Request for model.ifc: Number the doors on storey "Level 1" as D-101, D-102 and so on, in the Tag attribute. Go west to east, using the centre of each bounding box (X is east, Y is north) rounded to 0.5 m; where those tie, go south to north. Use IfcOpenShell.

First a look at what the model holds.

```python
import ifcopenshell
import ifcopenshell.util.element
import ifcopenshell.util.placement

model = ifcopenshell.open("model.ifc")
print(model.schema)
storey = next(s for s in model.by_type("IfcBuildingStorey") if s.Name == "Level 1")
doors = [e for e in ifcopenshell.util.element.get_decomposition(storey) if e.is_a("IfcDoor")]
for e in sorted(doors, key=lambda e: e.id()):
    origin = ifcopenshell.util.placement.get_local_placement(e.ObjectPlacement)[:3, 3]
    print(e.id(), e.Tag, e.Name, origin.round(2) + 0.0, sep=" | ")
```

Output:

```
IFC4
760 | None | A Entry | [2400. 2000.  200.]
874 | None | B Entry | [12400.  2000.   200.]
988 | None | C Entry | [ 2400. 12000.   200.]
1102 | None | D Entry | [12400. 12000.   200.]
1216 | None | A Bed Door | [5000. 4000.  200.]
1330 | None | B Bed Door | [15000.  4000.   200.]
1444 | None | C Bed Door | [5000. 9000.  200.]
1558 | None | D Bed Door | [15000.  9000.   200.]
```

```python
import ifcopenshell
import ifcopenshell.geom
import ifcopenshell.util.element
import ifcopenshell.util.shape

model = ifcopenshell.open("model.ifc")
settings = ifcopenshell.geom.settings()
settings.set("use-world-coords", True)


def centre(element):
    shape = ifcopenshell.geom.create_shape(settings, element)
    return ifcopenshell.util.shape.get_bbox_centroid(shape.geometry)


storey = next(s for s in model.by_type("IfcBuildingStorey") if s.Name == "Level 1")
doors = [e for e in ifcopenshell.util.element.get_decomposition(storey) if e.is_a("IfcDoor")]

# Insertion points can sit at a corner or the storey origin, so sort by the geometry (in metres).
centres = {e: centre(e) for e in doors}
doors.sort(key=lambda e: (round(centres[e][0] / 0.5), centres[e][1]))

for i, e in enumerate(doors, start=1):
    number = f"D-1{i:02d}"
    e.Tag = number
    print(e.id(), number)

model.write("model_edited.ifc")
```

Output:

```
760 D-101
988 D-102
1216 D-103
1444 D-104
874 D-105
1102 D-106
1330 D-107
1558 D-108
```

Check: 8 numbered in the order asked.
